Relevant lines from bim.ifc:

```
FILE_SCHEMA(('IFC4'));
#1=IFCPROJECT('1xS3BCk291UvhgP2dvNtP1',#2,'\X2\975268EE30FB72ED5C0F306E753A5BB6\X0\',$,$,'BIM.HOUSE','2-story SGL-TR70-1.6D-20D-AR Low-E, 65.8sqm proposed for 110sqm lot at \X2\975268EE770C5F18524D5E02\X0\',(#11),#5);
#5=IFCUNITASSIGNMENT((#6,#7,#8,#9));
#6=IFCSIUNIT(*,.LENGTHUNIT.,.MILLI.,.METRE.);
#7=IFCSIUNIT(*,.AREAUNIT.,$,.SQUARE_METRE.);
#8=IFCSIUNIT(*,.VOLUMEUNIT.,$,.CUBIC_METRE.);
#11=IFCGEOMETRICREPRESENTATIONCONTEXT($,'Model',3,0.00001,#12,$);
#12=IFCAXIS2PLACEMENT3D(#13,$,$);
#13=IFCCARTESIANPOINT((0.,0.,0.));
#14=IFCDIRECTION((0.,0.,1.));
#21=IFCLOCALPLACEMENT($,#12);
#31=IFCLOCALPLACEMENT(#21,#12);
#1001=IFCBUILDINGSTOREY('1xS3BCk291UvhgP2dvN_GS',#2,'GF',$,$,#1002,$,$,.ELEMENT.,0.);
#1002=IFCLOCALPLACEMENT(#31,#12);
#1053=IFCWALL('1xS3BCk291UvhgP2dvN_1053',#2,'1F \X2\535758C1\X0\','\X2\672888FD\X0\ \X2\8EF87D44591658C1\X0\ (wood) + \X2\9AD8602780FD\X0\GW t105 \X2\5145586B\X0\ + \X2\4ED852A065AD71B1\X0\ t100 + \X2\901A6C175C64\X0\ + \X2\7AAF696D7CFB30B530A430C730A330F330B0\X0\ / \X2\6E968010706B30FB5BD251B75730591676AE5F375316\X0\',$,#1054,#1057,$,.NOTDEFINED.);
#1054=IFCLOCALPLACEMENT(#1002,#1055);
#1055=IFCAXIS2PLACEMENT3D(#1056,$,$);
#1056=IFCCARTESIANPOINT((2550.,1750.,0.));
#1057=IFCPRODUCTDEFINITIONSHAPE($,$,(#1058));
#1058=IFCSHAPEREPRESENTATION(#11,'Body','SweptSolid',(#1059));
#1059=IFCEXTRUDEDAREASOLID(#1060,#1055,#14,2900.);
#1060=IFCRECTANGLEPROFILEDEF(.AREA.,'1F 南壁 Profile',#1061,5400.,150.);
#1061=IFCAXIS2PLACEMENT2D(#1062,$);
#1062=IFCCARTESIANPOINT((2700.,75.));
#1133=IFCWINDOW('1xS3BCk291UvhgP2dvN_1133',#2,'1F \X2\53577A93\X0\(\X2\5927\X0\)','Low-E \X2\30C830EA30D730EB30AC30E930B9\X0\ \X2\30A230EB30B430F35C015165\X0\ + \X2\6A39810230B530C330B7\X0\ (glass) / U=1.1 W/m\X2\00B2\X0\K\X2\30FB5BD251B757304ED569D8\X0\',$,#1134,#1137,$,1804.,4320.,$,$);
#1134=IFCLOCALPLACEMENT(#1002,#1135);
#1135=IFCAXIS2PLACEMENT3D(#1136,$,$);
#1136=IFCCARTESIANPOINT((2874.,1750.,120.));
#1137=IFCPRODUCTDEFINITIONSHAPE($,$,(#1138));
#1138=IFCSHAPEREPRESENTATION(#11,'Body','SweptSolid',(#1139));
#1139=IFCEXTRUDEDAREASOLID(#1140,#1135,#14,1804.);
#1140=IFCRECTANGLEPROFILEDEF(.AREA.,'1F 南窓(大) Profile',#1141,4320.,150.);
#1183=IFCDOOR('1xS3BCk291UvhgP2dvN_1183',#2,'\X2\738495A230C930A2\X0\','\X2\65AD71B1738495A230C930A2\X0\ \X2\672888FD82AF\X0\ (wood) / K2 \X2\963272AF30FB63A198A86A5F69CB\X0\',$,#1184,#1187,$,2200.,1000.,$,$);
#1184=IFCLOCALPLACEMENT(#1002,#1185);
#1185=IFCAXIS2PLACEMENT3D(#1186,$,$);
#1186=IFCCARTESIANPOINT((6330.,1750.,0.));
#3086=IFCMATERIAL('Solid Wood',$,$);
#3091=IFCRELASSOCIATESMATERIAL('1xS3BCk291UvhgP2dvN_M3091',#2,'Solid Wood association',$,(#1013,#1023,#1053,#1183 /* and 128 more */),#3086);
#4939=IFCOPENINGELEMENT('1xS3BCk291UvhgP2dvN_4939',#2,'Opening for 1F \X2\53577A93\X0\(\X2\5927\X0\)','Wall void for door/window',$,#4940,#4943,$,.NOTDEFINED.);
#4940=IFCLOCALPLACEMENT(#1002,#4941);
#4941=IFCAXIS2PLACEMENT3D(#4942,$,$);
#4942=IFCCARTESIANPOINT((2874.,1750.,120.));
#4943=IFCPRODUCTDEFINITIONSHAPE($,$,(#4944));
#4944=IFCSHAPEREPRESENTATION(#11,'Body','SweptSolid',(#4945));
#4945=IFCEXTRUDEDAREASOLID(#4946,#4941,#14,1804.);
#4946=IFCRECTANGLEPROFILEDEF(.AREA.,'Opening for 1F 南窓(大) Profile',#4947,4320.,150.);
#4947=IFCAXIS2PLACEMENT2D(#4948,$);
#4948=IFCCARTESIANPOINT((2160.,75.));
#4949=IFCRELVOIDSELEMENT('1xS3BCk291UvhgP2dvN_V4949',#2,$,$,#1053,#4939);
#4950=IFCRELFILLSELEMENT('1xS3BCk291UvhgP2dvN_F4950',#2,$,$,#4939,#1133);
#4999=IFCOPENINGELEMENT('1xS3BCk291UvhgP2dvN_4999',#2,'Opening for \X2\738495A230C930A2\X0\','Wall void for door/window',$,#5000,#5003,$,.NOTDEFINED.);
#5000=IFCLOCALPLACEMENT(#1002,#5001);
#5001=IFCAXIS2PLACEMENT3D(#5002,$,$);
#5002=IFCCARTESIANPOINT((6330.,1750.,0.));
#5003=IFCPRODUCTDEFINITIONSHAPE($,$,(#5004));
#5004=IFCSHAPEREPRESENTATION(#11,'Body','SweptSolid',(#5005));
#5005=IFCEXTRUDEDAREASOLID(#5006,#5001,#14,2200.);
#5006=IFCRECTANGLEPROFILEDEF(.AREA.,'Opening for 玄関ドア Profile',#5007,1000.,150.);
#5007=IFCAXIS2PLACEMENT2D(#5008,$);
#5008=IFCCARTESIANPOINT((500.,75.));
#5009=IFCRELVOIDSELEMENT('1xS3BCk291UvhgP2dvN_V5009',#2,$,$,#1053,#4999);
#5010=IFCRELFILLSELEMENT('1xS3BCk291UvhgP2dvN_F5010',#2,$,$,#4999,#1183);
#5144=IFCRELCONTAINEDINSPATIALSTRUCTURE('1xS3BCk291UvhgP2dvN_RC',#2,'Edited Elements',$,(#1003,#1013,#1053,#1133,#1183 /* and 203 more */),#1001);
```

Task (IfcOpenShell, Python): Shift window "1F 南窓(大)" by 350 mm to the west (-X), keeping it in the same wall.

```python
import ifcopenshell
import ifcopenshell.api.geometry
import ifcopenshell.util.placement
import ifcopenshell.util.unit

model = ifcopenshell.open("bim.ifc")
unit_scale = ifcopenshell.util.unit.calculate_unit_scale(model)

window = model.by_id(1133)
opening = window.FillsVoids[0].RelatingOpeningElement
wall = opening.VoidsElements[0].RelatingBuildingElement

wall_matrix = ifcopenshell.util.placement.get_local_placement(wall.ObjectPlacement)
shift = wall_matrix[:3, 0] * -0.35 / unit_scale
before = ifcopenshell.util.placement.get_local_placement(window.ObjectPlacement)[:3, 3].copy()

# The window is not placed relative to its opening, so move both.
for product in (opening, window):
    matrix = ifcopenshell.util.placement.get_local_placement(product.ObjectPlacement)
    matrix[:3, 3] += shift
    ifcopenshell.api.geometry.edit_object_placement(model, product=product, matrix=matrix, is_si=False)

after = ifcopenshell.util.placement.get_local_placement(window.ObjectPlacement)[:3, 3]
print("window moved by", (after - before).round(3) + 0.0)

model.write("bim_v2.ifc")
```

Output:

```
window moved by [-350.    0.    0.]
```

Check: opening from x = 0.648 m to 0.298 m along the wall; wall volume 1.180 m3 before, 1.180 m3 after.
